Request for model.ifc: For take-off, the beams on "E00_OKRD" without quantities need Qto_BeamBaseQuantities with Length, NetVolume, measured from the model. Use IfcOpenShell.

First a look at what the model holds.

```python
import ifcopenshell
import ifcopenshell.util.element
import ifcopenshell.util.unit

model = ifcopenshell.open("model.ifc")
print(model.schema)
for unit_type in ("LENGTHUNIT", "AREAUNIT", "VOLUMEUNIT"):
    print(unit_type, ifcopenshell.util.unit.calculate_unit_scale(model, unit_type))
storey = next(s for s in model.by_type("IfcBuildingStorey") if s.Name == "E00_OKRD")
beams = [e for e in ifcopenshell.util.element.get_decomposition(storey) if e.is_a("IfcBeam")]
for e in sorted(beams, key=lambda e: e.id()):
    print(e.id(), e.is_a(), e.Name, list(ifcopenshell.util.element.get_psets(e, qtos_only=True)), sep=" | ")
```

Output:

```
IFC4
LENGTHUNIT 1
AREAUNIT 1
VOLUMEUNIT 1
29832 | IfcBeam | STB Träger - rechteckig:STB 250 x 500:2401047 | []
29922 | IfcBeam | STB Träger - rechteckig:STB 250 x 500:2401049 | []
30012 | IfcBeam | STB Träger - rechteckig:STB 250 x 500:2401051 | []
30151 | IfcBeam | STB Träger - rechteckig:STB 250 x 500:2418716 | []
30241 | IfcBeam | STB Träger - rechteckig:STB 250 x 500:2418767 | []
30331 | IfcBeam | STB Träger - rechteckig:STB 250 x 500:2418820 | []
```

```python
import ifcopenshell
import ifcopenshell.api.pset
import ifcopenshell.geom
import ifcopenshell.util.element
import ifcopenshell.util.shape
import ifcopenshell.util.unit

model = ifcopenshell.open("model.ifc")
unit_scale = ifcopenshell.util.unit.calculate_unit_scale(model)
volume_scale = ifcopenshell.util.unit.calculate_unit_scale(model, "VOLUMEUNIT")
settings = ifcopenshell.geom.settings()

storey = next(s for s in model.by_type("IfcBuildingStorey") if s.Name == "E00_OKRD")
beams = [e for e in ifcopenshell.util.element.get_decomposition(storey) if e.is_a("IfcBeam")]

for e in sorted(beams, key=lambda e: e.id()):
    if ifcopenshell.util.element.get_psets(e, qtos_only=True, should_inherit=False):
        continue
    # Geometry comes back in metres, in the element's own axes.
    shape = ifcopenshell.geom.create_shape(settings, e)
    values = {
        "Length": ifcopenshell.util.shape.get_max_xyz(shape.geometry) / unit_scale,
        "NetVolume": ifcopenshell.util.shape.get_volume(shape.geometry) / volume_scale,
    }
    qto = ifcopenshell.api.pset.add_qto(model, product=e, name="Qto_BeamBaseQuantities")
    ifcopenshell.api.pset.edit_qto(model, qto=qto, properties=values)
    print(e.id(), {k: round(v, 3) for k, v in values.items()})

model.write("model_updated.ifc")
```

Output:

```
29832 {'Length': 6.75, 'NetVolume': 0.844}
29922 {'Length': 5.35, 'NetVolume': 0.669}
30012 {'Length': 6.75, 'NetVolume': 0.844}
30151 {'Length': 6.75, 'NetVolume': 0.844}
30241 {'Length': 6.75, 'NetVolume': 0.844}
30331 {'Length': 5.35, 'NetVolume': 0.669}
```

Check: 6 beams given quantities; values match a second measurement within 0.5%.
